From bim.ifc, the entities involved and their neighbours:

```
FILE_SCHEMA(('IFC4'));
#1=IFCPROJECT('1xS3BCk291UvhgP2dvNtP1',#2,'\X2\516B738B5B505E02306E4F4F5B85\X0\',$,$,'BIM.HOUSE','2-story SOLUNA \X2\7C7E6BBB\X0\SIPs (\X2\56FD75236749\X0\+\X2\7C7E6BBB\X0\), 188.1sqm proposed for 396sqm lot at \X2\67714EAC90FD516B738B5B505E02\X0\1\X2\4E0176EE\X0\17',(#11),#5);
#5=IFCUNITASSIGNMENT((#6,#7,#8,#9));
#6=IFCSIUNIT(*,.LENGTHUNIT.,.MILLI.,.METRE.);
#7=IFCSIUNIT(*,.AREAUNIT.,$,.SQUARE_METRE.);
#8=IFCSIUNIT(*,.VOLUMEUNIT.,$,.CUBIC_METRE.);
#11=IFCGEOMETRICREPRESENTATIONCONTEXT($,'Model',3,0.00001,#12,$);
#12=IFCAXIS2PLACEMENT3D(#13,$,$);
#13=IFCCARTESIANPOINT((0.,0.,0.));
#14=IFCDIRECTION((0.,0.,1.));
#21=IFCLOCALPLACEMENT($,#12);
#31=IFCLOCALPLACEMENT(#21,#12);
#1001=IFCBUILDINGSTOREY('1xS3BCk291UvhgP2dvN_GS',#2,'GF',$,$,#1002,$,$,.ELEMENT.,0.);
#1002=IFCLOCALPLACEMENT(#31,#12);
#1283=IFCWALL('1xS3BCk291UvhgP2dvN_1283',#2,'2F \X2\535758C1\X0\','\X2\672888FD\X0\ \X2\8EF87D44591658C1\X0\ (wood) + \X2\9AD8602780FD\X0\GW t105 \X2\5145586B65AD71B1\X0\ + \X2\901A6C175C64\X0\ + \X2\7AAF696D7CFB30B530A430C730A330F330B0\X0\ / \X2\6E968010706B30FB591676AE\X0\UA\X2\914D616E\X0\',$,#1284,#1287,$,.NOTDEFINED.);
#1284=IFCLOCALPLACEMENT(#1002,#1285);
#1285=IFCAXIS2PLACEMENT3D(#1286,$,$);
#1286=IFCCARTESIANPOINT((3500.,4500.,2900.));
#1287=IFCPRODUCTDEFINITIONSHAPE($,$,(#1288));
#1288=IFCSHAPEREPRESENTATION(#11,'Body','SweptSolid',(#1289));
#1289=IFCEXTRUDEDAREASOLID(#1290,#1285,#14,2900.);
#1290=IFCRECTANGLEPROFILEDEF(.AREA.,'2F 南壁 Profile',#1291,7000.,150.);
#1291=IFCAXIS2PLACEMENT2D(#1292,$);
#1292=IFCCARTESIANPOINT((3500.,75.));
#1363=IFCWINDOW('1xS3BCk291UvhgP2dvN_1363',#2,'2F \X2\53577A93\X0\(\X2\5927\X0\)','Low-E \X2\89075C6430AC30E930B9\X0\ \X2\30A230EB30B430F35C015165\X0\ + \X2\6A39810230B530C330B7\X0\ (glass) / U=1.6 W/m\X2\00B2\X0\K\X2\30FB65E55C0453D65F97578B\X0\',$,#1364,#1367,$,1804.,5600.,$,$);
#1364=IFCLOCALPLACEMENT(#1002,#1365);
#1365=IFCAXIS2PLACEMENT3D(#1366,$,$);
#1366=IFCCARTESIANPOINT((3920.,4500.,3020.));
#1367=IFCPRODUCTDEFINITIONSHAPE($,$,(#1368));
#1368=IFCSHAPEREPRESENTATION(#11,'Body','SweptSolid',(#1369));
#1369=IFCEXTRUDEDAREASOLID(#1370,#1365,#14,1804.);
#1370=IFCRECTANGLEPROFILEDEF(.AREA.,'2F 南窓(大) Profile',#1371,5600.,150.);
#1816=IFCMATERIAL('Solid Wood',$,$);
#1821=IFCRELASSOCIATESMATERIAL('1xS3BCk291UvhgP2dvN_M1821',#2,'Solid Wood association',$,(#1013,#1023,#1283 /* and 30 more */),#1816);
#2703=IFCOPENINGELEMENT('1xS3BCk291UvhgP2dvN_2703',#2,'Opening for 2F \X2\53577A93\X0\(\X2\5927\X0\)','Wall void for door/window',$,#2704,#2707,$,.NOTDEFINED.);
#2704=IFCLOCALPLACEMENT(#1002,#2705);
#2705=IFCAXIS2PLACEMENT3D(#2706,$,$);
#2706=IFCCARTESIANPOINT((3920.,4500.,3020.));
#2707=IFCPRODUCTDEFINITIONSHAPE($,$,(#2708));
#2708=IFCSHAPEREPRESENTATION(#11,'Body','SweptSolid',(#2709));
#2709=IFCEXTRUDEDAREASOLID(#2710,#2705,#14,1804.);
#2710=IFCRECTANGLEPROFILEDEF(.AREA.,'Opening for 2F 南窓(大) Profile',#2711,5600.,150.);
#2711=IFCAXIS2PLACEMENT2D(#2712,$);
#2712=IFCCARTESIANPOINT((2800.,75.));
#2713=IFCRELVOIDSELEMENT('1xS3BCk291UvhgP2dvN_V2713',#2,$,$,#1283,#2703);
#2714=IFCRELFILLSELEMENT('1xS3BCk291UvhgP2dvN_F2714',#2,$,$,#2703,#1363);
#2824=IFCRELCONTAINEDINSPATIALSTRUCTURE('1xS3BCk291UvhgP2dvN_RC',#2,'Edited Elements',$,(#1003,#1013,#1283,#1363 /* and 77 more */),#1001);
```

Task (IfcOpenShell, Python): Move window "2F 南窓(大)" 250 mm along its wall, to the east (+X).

```python
import ifcopenshell
import ifcopenshell.api.geometry
import ifcopenshell.util.placement
import ifcopenshell.util.unit

model = ifcopenshell.open("bim.ifc")
unit_scale = ifcopenshell.util.unit.calculate_unit_scale(model)

window = model.by_guid("1xS3BCk291UvhgP2dvN_1363")
opening = window.FillsVoids[0].RelatingOpeningElement
wall = opening.VoidsElements[0].RelatingBuildingElement

wall_matrix = ifcopenshell.util.placement.get_local_placement(wall.ObjectPlacement)
shift = wall_matrix[:3, 0] * 0.25 / unit_scale
before = ifcopenshell.util.placement.get_local_placement(window.ObjectPlacement)[:3, 3].copy()

# The window is not placed relative to its opening, so move both.
for product in (opening, window):
    matrix = ifcopenshell.util.placement.get_local_placement(product.ObjectPlacement)
    matrix[:3, 3] += shift
    ifcopenshell.api.geometry.edit_object_placement(model, product=product, matrix=matrix, is_si=False)

after = ifcopenshell.util.placement.get_local_placement(window.ObjectPlacement)[:3, 3]
print("window moved by", (after - before).round(3) + 0.0)

model.write("bim_rev.ifc")
```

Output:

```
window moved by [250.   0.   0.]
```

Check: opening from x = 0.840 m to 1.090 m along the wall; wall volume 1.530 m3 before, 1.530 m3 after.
